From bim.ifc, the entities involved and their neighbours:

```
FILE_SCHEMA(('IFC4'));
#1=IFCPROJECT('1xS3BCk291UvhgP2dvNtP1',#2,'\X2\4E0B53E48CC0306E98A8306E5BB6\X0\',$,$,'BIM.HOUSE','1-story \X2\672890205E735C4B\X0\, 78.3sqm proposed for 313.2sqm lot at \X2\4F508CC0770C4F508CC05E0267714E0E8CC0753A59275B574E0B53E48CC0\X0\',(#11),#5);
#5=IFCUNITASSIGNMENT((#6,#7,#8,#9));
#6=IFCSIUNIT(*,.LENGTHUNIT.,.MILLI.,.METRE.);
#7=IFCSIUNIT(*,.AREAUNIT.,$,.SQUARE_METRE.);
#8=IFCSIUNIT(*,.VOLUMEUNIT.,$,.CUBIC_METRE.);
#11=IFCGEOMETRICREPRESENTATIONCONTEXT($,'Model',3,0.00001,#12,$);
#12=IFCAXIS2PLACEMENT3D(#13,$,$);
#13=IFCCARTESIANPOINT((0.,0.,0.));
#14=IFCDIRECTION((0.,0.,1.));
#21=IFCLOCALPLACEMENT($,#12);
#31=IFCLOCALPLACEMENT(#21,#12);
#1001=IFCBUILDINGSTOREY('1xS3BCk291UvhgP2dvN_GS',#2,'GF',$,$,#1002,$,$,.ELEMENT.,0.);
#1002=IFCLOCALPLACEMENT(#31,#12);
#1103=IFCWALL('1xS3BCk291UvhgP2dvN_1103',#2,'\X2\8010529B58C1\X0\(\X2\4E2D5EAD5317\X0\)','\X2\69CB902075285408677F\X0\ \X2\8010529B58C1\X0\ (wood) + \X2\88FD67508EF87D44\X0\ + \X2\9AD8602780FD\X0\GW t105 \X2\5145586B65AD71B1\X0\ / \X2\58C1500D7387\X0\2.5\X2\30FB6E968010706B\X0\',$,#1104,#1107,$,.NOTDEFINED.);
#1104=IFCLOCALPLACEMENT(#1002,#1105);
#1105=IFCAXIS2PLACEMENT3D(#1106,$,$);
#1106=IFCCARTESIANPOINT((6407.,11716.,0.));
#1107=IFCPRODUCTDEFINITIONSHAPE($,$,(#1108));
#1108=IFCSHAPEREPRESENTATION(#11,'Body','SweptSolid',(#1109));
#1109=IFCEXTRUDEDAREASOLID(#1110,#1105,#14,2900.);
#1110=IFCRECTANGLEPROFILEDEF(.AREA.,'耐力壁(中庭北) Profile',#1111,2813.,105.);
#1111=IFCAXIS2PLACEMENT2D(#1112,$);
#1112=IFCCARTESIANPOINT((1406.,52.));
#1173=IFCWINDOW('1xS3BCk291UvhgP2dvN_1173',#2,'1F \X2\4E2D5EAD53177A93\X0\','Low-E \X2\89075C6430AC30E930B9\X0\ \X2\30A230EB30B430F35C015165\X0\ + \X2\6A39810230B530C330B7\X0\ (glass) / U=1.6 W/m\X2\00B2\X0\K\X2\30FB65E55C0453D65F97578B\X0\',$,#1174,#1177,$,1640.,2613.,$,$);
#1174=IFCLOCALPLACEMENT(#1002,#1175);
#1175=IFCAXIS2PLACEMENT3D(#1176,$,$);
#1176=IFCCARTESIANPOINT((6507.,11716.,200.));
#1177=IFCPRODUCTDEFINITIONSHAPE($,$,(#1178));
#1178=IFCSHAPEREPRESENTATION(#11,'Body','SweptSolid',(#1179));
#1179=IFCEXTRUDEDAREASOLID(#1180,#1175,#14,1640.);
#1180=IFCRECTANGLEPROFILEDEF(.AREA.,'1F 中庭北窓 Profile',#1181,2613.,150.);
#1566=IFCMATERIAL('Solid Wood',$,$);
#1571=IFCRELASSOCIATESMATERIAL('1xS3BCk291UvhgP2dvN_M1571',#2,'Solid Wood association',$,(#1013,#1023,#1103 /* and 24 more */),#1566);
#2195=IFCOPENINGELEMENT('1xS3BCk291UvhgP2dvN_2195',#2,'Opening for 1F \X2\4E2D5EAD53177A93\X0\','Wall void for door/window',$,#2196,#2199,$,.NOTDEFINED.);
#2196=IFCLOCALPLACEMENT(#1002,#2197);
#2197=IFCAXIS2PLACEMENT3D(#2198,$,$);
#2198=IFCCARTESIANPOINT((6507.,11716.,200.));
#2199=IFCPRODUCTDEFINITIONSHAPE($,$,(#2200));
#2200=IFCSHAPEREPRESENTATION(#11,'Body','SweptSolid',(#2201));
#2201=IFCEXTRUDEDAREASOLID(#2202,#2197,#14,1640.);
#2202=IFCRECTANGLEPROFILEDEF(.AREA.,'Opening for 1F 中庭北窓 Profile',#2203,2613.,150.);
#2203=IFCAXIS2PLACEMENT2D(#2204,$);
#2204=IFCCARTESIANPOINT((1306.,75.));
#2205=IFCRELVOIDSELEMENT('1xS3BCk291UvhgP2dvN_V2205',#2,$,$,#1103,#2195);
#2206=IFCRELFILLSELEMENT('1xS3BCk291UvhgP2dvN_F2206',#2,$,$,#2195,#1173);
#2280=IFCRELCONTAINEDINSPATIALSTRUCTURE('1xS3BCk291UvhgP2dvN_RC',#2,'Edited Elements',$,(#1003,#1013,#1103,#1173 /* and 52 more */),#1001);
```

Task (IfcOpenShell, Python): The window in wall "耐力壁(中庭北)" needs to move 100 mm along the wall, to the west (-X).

```python
import ifcopenshell
import ifcopenshell.api.geometry
import ifcopenshell.util.placement
import ifcopenshell.util.unit

model = ifcopenshell.open("bim.ifc")
unit_scale = ifcopenshell.util.unit.calculate_unit_scale(model)

window = model.by_id(1173)
opening = window.FillsVoids[0].RelatingOpeningElement
wall = opening.VoidsElements[0].RelatingBuildingElement

wall_matrix = ifcopenshell.util.placement.get_local_placement(wall.ObjectPlacement)
shift = wall_matrix[:3, 0] * -0.1 / unit_scale
before = ifcopenshell.util.placement.get_local_placement(window.ObjectPlacement)[:3, 3].copy()

# The window is not placed relative to its opening, so move both.
for product in (opening, window):
    matrix = ifcopenshell.util.placement.get_local_placement(product.ObjectPlacement)
    matrix[:3, 3] += shift
    ifcopenshell.api.geometry.edit_object_placement(model, product=product, matrix=matrix, is_si=False)

after = ifcopenshell.util.placement.get_local_placement(window.ObjectPlacement)[:3, 3]
print("window moved by", (after - before).round(3) + 0.0)

model.write("bim-out.ifc")
```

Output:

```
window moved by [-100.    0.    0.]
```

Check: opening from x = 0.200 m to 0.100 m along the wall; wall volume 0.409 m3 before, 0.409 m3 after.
